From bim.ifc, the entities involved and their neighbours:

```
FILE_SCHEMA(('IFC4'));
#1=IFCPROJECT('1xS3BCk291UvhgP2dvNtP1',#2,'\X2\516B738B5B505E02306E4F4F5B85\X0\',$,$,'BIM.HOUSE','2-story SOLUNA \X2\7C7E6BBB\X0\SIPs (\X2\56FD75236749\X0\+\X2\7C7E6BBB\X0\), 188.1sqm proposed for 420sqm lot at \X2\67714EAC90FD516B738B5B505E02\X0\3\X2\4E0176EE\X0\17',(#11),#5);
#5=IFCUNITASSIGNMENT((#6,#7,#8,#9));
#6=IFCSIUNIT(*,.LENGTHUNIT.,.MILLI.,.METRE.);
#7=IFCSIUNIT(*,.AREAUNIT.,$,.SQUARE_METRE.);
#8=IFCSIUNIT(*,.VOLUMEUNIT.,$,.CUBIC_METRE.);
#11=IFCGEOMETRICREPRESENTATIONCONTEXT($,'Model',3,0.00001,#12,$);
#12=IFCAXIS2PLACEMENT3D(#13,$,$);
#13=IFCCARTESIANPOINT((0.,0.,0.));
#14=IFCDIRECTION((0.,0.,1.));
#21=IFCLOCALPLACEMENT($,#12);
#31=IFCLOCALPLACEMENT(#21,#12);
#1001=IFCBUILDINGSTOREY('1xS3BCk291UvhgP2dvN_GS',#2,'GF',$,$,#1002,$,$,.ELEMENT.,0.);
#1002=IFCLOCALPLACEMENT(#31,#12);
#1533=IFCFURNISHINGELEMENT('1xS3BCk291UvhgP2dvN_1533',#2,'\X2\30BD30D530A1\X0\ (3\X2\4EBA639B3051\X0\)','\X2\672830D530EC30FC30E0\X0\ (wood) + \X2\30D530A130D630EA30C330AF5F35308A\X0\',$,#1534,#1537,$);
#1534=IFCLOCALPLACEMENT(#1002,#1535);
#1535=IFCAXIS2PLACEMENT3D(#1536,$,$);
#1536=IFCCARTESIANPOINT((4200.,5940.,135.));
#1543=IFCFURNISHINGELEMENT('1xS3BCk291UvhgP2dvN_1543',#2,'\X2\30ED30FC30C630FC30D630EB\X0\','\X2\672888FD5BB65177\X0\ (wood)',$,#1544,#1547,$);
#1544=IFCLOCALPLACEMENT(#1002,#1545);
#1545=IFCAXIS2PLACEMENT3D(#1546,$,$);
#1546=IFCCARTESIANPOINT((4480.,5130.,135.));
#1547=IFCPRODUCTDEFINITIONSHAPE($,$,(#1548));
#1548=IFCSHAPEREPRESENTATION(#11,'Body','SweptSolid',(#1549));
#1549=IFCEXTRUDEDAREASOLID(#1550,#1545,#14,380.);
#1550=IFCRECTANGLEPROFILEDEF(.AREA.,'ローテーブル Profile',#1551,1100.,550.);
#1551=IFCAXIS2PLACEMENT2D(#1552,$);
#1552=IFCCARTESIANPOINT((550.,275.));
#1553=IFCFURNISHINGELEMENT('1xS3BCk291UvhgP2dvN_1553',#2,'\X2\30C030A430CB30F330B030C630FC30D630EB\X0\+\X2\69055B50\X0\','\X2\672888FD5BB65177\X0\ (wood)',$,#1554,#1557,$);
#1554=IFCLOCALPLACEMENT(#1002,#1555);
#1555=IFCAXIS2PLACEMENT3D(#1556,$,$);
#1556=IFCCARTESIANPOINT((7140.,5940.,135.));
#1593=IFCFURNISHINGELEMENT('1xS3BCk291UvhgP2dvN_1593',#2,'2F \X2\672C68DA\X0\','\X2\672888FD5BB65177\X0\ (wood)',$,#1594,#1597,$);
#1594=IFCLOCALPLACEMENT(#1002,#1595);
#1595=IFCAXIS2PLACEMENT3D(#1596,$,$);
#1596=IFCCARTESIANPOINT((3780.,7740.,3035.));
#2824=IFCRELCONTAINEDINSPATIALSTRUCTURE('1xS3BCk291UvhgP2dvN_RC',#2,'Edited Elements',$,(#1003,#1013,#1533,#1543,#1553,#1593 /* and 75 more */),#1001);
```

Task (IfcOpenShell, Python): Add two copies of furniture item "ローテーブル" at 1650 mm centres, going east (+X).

```python
import numpy as np
import ifcopenshell
import ifcopenshell.api.geometry
import ifcopenshell.api.root
import ifcopenshell.util.element
import ifcopenshell.util.placement

model = ifcopenshell.open("bim.ifc")


def reuse_history(source, copy):
    """copy_class also copies each property set's owner history, people and application; keep the originals."""
    for rel in copy.IsDefinedBy:
        if rel.is_a("IfcRelDefinesByProperties") and (history := rel.RelatingPropertyDefinition.OwnerHistory):
            rel.RelatingPropertyDefinition.OwnerHistory = source.OwnerHistory
            ifcopenshell.util.element.remove_deep2(model, history)


source = model.by_guid("1xS3BCk291UvhgP2dvN_1543")
base = ifcopenshell.util.placement.get_local_placement(source.ObjectPlacement)
step = np.array([1.0, 0.0, 0.0]) * 1650.0

for i in range(1, 3):
    copy = ifcopenshell.api.root.copy_class(model, product=source)
    copy.Representation = ifcopenshell.util.element.copy_deep(
        model, source.Representation, exclude=["IfcGeometricRepresentationContext", "IfcRepresentationMap"]
    )
    reuse_history(source, copy)
    matrix = base.copy()
    matrix[:3, 3] += i * step
    print("added at", matrix[:3, 3].round(3) + 0.0)
    ifcopenshell.api.geometry.edit_object_placement(model, product=copy, matrix=matrix, is_si=False)

model.write("bim_edited.ifc")
```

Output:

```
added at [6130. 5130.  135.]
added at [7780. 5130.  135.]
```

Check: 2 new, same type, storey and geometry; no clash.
